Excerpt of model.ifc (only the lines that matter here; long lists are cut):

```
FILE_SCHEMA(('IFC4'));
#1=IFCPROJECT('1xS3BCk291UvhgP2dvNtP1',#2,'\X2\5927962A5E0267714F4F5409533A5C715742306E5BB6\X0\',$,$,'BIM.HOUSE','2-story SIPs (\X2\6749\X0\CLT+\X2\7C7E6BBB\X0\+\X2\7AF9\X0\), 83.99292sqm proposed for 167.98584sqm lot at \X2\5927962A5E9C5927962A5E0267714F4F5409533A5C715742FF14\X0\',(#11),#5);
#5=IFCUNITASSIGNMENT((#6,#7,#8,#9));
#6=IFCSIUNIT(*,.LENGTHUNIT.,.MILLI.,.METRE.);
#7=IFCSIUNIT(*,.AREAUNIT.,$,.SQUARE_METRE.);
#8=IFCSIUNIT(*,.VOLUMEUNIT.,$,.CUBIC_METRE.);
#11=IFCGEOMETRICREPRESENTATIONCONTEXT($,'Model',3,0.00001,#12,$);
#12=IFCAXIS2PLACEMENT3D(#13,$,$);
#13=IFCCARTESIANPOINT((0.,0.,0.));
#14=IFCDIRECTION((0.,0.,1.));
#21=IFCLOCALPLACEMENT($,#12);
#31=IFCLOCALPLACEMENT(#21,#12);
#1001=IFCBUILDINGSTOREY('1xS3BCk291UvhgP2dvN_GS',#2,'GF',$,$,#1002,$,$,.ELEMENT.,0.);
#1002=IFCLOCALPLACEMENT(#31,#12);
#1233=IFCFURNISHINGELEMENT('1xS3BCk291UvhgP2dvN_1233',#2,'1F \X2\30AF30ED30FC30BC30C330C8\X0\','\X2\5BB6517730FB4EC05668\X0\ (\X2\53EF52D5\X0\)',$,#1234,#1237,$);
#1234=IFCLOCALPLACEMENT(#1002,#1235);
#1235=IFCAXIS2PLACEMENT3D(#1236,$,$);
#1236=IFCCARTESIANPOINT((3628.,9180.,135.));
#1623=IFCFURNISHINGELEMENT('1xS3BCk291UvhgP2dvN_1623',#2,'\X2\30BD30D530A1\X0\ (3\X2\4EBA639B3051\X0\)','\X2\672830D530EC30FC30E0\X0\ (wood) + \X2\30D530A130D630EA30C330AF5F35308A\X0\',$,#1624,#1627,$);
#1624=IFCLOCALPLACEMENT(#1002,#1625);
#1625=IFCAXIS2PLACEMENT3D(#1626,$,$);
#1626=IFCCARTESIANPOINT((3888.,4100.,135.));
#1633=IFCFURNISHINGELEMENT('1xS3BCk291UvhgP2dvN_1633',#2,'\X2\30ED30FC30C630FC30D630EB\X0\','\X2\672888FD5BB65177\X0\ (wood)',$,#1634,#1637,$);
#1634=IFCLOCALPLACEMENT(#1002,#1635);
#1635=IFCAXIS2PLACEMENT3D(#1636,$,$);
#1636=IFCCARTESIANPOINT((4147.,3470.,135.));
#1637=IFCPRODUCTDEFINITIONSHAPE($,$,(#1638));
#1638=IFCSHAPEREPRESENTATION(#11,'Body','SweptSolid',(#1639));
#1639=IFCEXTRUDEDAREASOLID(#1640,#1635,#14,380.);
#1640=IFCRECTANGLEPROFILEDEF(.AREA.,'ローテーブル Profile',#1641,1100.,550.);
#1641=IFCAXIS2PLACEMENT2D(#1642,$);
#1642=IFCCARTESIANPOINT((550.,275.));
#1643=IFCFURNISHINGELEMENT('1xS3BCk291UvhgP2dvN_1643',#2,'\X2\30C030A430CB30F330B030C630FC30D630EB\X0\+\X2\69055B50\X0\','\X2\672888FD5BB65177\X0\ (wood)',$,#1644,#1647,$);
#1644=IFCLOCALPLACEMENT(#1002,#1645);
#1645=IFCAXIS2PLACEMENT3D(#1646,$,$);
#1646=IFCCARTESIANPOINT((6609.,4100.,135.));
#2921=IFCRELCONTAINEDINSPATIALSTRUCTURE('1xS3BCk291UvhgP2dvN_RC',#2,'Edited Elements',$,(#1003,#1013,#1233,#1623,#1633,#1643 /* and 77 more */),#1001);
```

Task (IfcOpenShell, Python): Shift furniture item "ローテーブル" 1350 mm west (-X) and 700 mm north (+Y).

```python
import ifcopenshell
import ifcopenshell.api.geometry
import ifcopenshell.util.placement

model = ifcopenshell.open("model.ifc")

item = model.by_guid("1xS3BCk291UvhgP2dvN_1633")
matrix = ifcopenshell.util.placement.get_local_placement(item.ObjectPlacement)
matrix[0, 3] -= 1350.0
matrix[1, 3] += 700.0
ifcopenshell.api.geometry.edit_object_placement(model, product=item, matrix=matrix, is_si=False)

print(ifcopenshell.util.placement.get_local_placement(item.ObjectPlacement).round(3) + 0.0)

model.write("model-out.ifc")
```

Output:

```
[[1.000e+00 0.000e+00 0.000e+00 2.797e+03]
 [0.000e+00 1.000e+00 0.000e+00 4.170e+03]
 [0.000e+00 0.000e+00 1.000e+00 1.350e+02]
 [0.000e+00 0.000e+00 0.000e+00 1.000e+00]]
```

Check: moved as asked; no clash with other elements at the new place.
